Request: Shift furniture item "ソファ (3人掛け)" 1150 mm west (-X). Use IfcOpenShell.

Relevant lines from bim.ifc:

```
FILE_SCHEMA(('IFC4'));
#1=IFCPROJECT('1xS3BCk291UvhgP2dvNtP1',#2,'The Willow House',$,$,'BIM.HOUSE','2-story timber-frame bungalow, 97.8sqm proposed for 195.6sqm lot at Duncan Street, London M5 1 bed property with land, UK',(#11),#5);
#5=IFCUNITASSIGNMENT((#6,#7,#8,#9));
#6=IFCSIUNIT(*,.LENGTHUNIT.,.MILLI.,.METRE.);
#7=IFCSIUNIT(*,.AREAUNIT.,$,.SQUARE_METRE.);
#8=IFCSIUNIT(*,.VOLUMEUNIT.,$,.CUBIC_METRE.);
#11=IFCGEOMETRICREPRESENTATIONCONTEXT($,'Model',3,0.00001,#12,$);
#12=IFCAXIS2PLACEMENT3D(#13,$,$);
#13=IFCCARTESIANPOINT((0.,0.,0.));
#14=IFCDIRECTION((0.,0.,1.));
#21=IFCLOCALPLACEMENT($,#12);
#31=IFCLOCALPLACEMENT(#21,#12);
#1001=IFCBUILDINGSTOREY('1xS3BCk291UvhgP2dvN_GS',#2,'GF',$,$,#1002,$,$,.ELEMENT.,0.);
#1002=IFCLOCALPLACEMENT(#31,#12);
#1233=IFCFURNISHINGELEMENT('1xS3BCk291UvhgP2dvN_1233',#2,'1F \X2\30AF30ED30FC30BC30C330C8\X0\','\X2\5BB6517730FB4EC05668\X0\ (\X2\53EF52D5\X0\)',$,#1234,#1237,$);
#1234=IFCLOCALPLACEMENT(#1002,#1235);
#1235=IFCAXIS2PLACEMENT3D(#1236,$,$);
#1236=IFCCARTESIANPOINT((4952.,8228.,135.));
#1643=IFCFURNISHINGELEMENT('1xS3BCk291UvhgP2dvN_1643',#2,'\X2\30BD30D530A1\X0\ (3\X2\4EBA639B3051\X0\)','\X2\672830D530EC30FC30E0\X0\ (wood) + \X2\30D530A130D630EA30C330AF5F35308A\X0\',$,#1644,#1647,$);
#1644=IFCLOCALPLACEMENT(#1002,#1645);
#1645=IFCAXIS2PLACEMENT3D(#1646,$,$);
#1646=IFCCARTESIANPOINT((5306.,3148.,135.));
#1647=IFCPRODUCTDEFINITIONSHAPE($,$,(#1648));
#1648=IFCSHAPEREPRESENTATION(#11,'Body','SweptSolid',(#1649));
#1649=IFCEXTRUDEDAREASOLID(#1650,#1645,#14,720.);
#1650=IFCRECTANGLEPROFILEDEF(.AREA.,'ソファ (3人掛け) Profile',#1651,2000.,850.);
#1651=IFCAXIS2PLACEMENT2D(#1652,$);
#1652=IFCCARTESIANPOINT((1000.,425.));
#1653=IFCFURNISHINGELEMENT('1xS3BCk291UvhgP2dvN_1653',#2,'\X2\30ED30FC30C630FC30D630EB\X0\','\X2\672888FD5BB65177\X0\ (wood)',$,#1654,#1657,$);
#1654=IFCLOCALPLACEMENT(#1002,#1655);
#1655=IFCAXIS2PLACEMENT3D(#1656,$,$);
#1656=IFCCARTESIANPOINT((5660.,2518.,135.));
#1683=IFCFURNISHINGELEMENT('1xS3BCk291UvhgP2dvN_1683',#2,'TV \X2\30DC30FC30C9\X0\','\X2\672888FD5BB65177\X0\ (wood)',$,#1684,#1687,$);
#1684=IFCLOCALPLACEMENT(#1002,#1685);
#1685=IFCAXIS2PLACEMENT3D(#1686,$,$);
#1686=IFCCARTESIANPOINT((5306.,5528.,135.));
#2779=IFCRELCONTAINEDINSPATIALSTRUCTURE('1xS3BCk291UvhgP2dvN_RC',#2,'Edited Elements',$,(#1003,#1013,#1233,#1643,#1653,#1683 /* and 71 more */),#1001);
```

```python
import ifcopenshell
import ifcopenshell.api.geometry
import ifcopenshell.util.placement

model = ifcopenshell.open("bim.ifc")

item = model.by_guid("1xS3BCk291UvhgP2dvN_1643")
matrix = ifcopenshell.util.placement.get_local_placement(item.ObjectPlacement)
matrix[0, 3] -= 1150.0
ifcopenshell.api.geometry.edit_object_placement(model, product=item, matrix=matrix, is_si=False)

print(ifcopenshell.util.placement.get_local_placement(item.ObjectPlacement).round(3) + 0.0)

model.write("bim-out.ifc")
```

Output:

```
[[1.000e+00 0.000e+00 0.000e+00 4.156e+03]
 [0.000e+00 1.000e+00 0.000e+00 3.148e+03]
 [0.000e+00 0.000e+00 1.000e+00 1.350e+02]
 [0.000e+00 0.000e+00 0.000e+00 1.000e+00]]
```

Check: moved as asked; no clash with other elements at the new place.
